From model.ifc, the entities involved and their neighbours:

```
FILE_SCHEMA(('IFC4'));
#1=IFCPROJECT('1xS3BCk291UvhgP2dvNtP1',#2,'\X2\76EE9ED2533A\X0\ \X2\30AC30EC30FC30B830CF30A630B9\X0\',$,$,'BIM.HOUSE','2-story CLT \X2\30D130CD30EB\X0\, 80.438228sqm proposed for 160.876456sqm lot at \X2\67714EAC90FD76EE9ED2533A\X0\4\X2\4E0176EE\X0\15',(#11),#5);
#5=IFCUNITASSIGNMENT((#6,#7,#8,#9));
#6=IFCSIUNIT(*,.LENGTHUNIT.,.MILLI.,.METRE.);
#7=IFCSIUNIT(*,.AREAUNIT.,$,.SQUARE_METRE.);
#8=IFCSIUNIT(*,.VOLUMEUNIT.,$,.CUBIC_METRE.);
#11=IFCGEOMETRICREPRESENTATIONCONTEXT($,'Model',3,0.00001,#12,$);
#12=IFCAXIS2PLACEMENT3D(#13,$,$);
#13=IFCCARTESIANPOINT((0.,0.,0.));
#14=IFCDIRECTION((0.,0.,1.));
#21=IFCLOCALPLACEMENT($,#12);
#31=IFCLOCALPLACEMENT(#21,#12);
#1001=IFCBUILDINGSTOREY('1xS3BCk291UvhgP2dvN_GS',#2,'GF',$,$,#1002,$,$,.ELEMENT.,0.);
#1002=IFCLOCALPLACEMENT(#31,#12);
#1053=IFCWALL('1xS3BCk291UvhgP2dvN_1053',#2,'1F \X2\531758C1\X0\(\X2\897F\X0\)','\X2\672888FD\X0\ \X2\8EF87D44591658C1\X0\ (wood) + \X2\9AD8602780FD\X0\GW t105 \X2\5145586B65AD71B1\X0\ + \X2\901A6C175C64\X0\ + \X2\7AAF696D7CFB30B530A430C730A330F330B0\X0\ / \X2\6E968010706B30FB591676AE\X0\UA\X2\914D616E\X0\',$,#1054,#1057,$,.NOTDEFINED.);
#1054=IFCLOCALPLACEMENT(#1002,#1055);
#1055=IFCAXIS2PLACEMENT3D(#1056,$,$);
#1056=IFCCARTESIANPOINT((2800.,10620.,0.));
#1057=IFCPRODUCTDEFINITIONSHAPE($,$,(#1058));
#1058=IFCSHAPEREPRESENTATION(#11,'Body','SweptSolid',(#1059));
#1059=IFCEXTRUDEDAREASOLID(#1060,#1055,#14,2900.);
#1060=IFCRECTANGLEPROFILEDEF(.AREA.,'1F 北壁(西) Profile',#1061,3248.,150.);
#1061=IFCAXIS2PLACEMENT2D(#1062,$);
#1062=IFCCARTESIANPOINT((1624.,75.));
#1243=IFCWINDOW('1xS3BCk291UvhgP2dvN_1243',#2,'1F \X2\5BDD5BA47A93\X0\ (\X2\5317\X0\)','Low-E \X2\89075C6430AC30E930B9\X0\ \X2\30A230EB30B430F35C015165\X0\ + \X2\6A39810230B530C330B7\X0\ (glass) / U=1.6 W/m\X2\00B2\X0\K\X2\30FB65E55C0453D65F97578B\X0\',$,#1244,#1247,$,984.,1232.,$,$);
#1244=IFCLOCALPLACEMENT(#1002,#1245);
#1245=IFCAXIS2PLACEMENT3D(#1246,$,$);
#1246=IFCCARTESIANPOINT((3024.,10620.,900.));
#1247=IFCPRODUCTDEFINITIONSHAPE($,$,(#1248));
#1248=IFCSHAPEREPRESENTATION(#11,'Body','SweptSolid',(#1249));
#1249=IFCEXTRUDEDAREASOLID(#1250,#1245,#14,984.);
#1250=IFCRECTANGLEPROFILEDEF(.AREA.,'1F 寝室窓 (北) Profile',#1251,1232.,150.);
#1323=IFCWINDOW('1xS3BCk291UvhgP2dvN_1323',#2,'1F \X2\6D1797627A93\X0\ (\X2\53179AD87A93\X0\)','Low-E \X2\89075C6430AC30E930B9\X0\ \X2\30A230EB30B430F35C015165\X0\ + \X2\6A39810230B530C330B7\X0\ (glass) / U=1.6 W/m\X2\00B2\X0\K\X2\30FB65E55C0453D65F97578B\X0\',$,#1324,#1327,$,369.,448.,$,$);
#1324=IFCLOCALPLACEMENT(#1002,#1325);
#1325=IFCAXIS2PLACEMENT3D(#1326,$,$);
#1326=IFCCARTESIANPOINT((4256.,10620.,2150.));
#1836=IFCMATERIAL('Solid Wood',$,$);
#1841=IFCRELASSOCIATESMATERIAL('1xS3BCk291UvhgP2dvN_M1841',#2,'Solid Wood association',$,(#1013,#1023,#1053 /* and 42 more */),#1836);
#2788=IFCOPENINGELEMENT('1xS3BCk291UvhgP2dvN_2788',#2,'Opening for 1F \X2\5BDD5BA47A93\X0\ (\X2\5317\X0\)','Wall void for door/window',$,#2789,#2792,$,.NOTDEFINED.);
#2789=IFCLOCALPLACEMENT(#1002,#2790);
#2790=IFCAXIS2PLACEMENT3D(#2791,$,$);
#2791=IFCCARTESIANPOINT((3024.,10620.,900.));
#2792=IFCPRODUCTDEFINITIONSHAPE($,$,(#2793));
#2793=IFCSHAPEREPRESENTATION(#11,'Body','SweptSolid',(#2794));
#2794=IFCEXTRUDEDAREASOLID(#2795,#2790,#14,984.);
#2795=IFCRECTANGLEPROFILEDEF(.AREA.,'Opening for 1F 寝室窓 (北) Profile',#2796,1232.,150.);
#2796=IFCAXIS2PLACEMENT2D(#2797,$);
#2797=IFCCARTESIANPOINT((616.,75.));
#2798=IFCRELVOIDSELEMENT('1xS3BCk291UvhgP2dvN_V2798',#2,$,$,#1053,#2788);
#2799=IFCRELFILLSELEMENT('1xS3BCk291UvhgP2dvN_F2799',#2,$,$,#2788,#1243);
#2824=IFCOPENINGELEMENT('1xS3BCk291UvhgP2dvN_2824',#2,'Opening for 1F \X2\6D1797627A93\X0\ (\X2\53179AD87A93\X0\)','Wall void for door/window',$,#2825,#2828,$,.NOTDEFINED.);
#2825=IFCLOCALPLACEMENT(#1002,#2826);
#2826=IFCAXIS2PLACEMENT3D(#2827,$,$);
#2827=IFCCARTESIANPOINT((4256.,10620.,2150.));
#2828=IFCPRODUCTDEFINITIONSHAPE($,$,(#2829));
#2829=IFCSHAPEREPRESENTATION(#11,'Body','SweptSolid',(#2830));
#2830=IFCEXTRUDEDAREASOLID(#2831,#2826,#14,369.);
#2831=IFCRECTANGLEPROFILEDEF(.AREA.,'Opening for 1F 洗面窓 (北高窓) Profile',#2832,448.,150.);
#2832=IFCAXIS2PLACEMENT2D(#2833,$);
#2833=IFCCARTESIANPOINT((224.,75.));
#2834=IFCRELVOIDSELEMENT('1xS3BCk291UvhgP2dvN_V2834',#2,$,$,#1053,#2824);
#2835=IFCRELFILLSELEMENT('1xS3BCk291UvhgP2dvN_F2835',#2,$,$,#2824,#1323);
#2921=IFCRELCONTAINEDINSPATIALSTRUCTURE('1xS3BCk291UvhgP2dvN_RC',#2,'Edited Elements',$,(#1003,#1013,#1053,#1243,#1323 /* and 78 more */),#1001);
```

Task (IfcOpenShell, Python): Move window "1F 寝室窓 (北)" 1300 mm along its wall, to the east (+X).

```python
import ifcopenshell
import ifcopenshell.api.geometry
import ifcopenshell.util.placement

model = ifcopenshell.open("model.ifc")

window = model.by_guid("1xS3BCk291UvhgP2dvN_1243")
opening = window.FillsVoids[0].RelatingOpeningElement
wall = opening.VoidsElements[0].RelatingBuildingElement

wall_matrix = ifcopenshell.util.placement.get_local_placement(wall.ObjectPlacement)
shift = wall_matrix[:3, 0] * 1300.0
before = ifcopenshell.util.placement.get_local_placement(window.ObjectPlacement)[:3, 3].copy()

# The window is not placed relative to its opening, so move both.
for product in (opening, window):
    matrix = ifcopenshell.util.placement.get_local_placement(product.ObjectPlacement)
    matrix[:3, 3] += shift
    ifcopenshell.api.geometry.edit_object_placement(model, product=product, matrix=matrix, is_si=False)

after = ifcopenshell.util.placement.get_local_placement(window.ObjectPlacement)[:3, 3]
print("window moved by", (after - before).round(3) + 0.0)

model.write("model_updated.ifc")
```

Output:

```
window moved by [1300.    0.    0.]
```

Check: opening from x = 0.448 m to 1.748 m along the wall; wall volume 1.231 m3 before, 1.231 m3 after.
